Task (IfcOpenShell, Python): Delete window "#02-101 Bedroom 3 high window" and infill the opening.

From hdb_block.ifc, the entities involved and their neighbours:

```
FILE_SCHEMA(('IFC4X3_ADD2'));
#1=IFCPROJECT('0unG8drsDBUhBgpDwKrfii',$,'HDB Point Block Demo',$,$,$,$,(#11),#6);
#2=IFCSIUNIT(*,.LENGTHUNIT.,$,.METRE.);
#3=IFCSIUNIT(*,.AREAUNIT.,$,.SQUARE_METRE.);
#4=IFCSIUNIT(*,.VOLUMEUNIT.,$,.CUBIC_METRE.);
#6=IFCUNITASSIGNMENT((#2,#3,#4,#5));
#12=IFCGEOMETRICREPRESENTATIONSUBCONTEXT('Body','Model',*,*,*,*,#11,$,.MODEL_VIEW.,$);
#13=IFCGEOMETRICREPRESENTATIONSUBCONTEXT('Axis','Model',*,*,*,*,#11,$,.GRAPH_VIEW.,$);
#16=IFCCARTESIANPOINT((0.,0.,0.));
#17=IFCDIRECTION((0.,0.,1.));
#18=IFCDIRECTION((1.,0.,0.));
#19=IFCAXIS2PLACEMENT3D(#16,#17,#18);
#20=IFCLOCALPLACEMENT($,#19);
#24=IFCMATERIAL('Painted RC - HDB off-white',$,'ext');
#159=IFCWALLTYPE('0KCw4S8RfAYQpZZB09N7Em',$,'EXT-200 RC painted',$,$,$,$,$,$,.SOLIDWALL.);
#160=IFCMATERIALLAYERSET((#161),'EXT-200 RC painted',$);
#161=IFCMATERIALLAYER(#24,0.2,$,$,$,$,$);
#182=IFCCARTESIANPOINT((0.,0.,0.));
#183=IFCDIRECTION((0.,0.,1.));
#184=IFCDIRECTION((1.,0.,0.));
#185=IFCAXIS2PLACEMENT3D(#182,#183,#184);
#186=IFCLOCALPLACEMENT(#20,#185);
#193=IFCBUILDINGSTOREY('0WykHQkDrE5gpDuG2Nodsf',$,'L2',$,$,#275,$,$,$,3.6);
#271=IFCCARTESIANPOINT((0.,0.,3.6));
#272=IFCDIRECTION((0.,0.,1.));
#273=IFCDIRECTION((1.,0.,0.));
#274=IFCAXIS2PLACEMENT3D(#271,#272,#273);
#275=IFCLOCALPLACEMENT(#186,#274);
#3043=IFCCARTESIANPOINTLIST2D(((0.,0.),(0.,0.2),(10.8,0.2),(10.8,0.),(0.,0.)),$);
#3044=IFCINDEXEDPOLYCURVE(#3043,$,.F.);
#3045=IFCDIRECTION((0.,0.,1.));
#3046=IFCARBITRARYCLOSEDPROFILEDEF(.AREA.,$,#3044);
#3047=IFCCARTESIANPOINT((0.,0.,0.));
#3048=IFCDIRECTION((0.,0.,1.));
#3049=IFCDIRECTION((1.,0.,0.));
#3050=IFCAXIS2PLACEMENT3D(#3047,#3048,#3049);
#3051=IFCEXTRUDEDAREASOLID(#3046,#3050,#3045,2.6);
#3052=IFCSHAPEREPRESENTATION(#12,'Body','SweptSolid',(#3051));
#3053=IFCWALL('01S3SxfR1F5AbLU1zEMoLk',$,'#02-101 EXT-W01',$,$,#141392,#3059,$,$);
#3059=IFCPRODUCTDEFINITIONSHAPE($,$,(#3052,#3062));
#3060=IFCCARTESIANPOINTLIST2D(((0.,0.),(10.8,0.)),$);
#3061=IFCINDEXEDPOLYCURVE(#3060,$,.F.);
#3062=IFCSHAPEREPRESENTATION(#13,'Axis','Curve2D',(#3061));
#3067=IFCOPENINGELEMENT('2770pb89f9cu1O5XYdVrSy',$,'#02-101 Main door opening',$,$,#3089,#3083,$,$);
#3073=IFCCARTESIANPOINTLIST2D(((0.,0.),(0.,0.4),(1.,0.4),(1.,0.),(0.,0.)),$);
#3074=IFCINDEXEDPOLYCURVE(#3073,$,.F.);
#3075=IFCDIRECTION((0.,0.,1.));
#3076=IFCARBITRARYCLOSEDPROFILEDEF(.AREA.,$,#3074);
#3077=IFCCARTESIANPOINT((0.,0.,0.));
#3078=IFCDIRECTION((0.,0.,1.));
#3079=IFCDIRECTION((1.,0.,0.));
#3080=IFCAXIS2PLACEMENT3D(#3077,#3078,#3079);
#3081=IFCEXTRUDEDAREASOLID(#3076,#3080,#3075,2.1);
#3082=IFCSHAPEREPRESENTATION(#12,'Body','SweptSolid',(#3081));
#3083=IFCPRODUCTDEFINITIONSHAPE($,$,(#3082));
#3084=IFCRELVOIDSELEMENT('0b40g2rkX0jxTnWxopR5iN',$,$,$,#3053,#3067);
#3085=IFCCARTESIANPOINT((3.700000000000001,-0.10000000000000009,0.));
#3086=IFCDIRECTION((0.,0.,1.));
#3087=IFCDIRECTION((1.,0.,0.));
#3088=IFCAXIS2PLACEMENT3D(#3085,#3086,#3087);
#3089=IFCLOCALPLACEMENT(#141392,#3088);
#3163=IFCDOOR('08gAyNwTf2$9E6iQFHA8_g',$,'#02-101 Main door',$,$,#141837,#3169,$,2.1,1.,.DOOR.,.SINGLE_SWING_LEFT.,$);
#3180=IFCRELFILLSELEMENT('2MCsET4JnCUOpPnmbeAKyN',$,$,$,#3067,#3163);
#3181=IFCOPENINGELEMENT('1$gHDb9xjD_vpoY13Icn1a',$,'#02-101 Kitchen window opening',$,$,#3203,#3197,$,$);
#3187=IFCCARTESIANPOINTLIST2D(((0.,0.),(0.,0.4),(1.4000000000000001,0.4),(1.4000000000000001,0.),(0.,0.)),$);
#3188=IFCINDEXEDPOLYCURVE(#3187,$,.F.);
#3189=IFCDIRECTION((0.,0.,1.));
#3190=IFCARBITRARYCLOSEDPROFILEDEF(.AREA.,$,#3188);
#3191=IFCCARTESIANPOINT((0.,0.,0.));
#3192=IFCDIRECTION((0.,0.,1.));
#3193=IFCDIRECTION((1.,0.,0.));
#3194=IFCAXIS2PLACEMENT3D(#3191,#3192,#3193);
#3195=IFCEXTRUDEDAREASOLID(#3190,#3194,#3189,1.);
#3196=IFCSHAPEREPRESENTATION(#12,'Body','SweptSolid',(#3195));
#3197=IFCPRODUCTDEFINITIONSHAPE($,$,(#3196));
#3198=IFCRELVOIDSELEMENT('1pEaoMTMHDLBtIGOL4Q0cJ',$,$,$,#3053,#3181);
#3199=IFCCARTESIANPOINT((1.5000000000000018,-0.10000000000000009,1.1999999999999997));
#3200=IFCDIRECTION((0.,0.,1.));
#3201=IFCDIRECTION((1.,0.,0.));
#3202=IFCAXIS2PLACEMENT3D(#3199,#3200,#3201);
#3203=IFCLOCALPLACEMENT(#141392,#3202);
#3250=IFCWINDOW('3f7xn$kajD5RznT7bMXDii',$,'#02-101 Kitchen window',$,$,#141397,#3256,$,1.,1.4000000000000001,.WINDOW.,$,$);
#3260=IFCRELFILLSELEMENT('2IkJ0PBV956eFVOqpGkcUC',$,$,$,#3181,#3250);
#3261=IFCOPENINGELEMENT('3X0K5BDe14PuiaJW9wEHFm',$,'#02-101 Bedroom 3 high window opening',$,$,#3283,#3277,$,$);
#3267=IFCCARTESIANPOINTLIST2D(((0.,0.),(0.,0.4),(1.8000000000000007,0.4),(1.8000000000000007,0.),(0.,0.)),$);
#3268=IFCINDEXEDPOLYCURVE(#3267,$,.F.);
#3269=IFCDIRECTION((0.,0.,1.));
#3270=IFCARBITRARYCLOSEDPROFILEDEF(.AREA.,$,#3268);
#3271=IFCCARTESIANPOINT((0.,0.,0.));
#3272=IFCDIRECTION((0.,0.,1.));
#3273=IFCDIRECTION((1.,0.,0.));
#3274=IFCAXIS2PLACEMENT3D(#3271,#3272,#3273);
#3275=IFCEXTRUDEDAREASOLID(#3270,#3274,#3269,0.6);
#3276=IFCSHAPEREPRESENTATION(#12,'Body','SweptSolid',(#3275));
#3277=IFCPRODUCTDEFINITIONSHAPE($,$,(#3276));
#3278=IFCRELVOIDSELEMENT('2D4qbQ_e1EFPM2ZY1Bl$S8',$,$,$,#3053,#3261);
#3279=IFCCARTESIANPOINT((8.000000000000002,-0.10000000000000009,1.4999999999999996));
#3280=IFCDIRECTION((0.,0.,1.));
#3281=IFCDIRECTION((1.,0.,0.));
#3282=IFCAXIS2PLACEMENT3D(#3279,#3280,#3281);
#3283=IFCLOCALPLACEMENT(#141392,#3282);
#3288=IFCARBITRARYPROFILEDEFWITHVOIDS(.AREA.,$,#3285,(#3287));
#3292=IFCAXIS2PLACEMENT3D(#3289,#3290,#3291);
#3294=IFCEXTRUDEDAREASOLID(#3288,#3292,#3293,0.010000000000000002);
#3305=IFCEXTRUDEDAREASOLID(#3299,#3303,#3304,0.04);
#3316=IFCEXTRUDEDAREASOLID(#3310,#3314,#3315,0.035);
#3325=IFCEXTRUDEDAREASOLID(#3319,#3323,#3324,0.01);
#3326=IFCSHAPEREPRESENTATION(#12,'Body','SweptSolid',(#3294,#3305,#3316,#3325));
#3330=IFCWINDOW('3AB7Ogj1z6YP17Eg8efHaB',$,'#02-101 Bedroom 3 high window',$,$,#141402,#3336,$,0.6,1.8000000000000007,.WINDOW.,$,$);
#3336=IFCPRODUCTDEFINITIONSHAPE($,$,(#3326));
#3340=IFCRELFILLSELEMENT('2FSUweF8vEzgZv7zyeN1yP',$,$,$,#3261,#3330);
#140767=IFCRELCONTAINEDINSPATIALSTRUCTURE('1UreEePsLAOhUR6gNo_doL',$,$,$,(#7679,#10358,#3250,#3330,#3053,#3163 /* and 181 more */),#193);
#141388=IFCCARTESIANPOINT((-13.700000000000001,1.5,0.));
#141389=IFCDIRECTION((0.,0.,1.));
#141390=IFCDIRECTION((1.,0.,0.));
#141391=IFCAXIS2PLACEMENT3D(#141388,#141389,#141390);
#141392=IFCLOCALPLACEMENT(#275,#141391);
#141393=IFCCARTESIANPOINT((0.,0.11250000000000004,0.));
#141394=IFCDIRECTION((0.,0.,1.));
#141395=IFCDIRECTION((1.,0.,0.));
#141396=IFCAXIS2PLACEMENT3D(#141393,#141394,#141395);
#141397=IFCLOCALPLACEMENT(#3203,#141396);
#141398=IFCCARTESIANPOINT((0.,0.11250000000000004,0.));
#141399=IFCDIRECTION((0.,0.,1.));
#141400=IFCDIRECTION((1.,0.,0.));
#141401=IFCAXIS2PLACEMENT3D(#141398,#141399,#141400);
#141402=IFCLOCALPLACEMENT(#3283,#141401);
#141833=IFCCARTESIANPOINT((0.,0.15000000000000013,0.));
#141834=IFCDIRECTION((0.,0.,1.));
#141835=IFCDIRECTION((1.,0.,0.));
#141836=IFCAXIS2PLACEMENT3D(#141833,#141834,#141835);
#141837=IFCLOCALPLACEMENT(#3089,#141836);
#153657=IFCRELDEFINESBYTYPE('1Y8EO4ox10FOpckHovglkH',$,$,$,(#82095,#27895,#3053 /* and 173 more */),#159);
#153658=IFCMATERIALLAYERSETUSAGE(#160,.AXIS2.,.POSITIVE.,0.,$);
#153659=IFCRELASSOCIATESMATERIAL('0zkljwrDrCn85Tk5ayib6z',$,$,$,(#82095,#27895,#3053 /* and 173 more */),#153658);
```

```python
import ifcopenshell
import ifcopenshell.api.feature
import ifcopenshell.api.root
import ifcopenshell.geom
import ifcopenshell.util.shape

model = ifcopenshell.open("hdb_block.ifc")
settings = ifcopenshell.geom.settings()


def volume(element):
    """Net volume in cubic metres, openings subtracted."""
    shape = ifcopenshell.geom.create_shape(settings, element)
    return ifcopenshell.util.shape.get_volume(shape.geometry)


window = model.by_guid("3AB7Ogj1z6YP17Eg8efHaB")
opening = window.FillsVoids[0].RelatingOpeningElement
wall = opening.VoidsElements[0].RelatingBuildingElement
before = volume(wall)

ifcopenshell.api.root.remove_product(model, product=window)
ifcopenshell.api.feature.remove_feature(model, feature=opening)

after = volume(wall)

print(f"wall volume {before:.3f} -> {after:.3f} m3")

model.write("hdb_block_v2.ifc")
```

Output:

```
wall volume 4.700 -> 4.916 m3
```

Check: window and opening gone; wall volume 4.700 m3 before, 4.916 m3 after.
